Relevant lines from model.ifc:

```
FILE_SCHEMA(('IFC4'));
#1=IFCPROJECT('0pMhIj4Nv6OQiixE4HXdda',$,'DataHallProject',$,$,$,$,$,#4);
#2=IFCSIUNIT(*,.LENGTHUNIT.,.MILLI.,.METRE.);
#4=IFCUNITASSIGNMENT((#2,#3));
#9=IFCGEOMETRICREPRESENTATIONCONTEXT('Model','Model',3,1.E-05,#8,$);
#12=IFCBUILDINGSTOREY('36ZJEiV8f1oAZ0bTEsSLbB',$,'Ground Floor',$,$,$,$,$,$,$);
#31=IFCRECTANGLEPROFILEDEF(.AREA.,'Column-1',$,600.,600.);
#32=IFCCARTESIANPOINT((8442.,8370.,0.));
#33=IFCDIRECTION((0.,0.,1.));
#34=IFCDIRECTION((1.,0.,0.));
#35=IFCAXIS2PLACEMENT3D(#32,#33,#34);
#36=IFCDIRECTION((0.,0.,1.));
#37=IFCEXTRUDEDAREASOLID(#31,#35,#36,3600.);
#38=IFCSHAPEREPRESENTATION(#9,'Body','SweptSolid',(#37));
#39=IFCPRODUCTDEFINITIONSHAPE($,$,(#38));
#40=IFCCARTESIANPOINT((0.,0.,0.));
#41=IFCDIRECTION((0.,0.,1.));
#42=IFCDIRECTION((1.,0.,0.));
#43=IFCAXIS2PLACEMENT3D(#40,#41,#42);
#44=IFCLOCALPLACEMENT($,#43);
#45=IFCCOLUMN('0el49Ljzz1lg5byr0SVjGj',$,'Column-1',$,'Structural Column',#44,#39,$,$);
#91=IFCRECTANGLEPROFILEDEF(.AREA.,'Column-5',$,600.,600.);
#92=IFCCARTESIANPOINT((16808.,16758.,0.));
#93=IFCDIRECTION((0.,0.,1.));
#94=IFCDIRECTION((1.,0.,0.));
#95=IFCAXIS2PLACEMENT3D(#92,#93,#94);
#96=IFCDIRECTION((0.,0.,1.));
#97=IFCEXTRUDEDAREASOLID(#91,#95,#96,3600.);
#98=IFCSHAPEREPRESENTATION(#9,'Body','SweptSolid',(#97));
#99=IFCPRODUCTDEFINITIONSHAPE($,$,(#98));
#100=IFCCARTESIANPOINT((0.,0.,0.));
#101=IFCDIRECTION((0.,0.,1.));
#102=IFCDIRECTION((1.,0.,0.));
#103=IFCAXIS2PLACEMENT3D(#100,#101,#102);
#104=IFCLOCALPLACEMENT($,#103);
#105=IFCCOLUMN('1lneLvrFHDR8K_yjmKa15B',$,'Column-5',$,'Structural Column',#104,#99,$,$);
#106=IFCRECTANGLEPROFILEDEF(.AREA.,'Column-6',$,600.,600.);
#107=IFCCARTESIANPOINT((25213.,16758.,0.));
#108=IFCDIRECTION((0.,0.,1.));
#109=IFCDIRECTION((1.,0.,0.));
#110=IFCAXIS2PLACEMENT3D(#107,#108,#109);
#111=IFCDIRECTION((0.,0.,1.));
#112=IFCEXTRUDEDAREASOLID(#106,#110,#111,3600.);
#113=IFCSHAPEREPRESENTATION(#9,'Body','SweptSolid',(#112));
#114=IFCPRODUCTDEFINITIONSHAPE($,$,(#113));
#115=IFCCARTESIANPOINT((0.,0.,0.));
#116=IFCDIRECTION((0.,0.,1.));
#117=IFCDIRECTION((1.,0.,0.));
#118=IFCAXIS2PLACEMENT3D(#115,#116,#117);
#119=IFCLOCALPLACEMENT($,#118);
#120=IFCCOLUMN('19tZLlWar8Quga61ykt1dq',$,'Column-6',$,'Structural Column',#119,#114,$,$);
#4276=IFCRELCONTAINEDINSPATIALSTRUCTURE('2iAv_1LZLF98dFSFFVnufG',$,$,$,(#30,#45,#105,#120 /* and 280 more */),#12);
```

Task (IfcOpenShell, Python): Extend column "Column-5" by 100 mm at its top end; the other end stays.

```python
import ifcopenshell

model = ifcopenshell.open("model.ifc")

member = model.by_guid("1lneLvrFHDR8K_yjmKa15B")
change = 100.0

# The extrusion runs towards the end named, so only its depth changes.
body = next(r for r in member.Representation.Representations if r.RepresentationIdentifier == "Body")
solid = body.Items[0]
old_length = solid.Depth
solid.Depth += change

print(f"length {old_length:g} -> {solid.Depth:g}")

model.write("model_updated.ifc")
```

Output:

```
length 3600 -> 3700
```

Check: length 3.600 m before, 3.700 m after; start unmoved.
